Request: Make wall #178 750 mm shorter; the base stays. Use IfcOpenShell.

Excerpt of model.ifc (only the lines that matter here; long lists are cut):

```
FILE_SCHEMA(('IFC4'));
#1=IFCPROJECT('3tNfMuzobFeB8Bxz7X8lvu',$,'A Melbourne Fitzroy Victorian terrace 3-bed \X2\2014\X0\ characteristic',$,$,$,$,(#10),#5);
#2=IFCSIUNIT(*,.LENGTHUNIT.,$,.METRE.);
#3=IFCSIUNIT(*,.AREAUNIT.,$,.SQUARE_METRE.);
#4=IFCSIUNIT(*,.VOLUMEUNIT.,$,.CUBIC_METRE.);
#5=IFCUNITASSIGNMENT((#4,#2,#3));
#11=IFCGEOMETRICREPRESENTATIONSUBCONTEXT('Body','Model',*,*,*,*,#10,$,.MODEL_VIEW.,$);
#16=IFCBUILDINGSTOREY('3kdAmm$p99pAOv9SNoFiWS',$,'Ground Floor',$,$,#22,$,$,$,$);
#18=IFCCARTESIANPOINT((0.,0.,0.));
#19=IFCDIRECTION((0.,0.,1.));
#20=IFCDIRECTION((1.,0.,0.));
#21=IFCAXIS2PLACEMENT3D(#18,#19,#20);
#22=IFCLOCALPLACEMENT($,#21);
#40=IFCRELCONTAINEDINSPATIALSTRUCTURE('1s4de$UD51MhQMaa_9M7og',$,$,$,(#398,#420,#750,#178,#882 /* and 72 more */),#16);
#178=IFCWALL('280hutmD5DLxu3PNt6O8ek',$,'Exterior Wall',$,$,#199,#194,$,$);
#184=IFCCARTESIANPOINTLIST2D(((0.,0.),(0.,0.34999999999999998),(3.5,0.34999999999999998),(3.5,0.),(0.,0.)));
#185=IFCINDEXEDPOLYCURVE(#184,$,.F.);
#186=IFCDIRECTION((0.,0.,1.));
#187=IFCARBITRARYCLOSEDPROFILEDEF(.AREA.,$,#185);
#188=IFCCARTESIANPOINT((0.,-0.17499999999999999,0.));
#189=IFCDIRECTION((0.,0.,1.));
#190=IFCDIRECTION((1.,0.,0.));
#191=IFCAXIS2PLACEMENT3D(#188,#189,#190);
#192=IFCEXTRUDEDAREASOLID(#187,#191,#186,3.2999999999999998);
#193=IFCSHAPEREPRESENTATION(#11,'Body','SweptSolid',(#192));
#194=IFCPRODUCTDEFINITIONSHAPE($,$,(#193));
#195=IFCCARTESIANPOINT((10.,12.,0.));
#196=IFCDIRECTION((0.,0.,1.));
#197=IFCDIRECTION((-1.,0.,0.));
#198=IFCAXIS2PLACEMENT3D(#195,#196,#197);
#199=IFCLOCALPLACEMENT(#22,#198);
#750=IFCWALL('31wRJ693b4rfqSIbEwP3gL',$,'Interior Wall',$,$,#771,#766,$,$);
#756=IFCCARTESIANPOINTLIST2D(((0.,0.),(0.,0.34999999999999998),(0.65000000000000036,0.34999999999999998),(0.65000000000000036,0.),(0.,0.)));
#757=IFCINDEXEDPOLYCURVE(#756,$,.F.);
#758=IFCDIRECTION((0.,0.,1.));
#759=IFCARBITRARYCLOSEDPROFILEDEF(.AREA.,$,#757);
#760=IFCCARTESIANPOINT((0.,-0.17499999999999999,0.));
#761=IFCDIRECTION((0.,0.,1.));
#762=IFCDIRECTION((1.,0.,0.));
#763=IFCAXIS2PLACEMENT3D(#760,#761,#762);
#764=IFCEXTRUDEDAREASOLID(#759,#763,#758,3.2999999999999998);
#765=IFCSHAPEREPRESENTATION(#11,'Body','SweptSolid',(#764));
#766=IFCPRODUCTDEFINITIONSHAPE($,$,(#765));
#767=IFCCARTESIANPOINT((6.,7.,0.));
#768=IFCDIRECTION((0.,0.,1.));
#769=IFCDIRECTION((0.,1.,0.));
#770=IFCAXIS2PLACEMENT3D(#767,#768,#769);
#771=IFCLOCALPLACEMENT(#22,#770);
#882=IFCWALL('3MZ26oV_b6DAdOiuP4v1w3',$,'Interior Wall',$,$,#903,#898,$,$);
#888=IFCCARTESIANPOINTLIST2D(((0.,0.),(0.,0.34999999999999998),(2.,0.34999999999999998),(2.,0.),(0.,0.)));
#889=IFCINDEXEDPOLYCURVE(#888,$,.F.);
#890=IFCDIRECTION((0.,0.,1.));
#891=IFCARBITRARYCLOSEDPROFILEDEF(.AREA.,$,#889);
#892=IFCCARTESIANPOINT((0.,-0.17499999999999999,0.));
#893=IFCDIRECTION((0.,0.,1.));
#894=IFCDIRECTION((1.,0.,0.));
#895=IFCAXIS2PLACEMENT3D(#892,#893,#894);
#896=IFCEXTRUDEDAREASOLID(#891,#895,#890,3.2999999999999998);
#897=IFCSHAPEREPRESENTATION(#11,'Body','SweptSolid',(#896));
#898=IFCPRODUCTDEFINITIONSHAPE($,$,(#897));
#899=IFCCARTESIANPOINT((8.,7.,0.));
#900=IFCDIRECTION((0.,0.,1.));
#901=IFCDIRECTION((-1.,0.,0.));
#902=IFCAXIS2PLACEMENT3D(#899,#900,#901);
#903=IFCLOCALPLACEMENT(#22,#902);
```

```python
import ifcopenshell
import ifcopenshell.geom
import ifcopenshell.util.representation
import ifcopenshell.util.shape
import ifcopenshell.util.unit

model = ifcopenshell.open("model.ifc")
unit_scale = ifcopenshell.util.unit.calculate_unit_scale(model)
settings = ifcopenshell.geom.settings()


def volume(element):
    """Net volume in cubic metres, openings subtracted."""
    shape = ifcopenshell.geom.create_shape(settings, element)
    return ifcopenshell.util.shape.get_volume(shape.geometry)


wall = model.by_id(178)
before = volume(wall)

body = ifcopenshell.util.representation.get_representation(wall, "Model", "Body")
solid = body.Items[0]
old_height = solid.Depth
solid.Depth -= 0.75 / unit_scale
after = volume(wall)

print(f"height {old_height:g} -> {solid.Depth:g}, volume {before:.3f} -> {after:.3f} m3")

model.write("model_updated.ifc")
```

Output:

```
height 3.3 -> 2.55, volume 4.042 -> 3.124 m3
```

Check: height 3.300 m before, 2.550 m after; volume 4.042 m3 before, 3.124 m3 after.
